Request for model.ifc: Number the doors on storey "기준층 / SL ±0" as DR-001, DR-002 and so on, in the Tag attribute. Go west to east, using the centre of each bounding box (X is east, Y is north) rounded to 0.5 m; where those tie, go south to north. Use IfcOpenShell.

First a look at what the model holds.

```python
import ifcopenshell
import ifcopenshell.util.element
import ifcopenshell.util.placement

model = ifcopenshell.open("model.ifc")
print(model.schema)
storey = next(s for s in model.by_type("IfcBuildingStorey") if s.Name == "기준층 / SL ±0")
doors = [e for e in ifcopenshell.util.element.get_decomposition(storey) if e.is_a("IfcDoor")]
for e in sorted(doors, key=lambda e: e.id()):
    origin = ifcopenshell.util.placement.get_local_placement(e.ObjectPlacement)[:3, 3]
    print(e.id(), e.Tag, e.Name, origin.round(2) + 0.0, sep=" | ")
```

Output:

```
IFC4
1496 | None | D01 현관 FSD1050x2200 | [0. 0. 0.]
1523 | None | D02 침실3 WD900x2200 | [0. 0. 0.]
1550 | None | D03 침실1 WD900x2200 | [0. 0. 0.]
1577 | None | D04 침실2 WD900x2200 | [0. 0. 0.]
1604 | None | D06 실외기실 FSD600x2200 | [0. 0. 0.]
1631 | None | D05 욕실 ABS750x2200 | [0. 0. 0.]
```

```python
import ifcopenshell
import ifcopenshell.geom
import ifcopenshell.util.element
import ifcopenshell.util.shape

model = ifcopenshell.open("model.ifc")
settings = ifcopenshell.geom.settings()
settings.set("use-world-coords", True)


def centre(element):
    shape = ifcopenshell.geom.create_shape(settings, element)
    return ifcopenshell.util.shape.get_bbox_centroid(shape.geometry)


storey = next(s for s in model.by_type("IfcBuildingStorey") if s.Name == "기준층 / SL ±0")
doors = [e for e in ifcopenshell.util.element.get_decomposition(storey) if e.is_a("IfcDoor")]

# Insertion points can sit at a corner or the storey origin, so sort by the geometry (in metres).
centres = {e: centre(e) for e in doors}
doors.sort(key=lambda e: (round(centres[e][0] / 0.5), centres[e][1]))

for i, e in enumerate(doors, start=1):
    number = f"DR-0{i:02d}"
    e.Tag = number
    print(e.id(), number)

model.write("model_edited.ifc")
```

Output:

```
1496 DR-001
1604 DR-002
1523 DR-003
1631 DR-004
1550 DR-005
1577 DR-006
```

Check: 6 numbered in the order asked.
